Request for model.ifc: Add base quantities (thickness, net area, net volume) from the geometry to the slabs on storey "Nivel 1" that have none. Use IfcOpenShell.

First a look at what the model holds.

```python
import ifcopenshell
import ifcopenshell.util.element
import ifcopenshell.util.unit

model = ifcopenshell.open("model.ifc")
print(model.schema)
for unit_type in ("LENGTHUNIT", "AREAUNIT", "VOLUMEUNIT"):
    print(unit_type, ifcopenshell.util.unit.calculate_unit_scale(model, unit_type))
storey = next(s for s in model.by_type("IfcBuildingStorey") if s.Name == "Nivel 1")
slabs = [e for e in ifcopenshell.util.element.get_decomposition(storey) if e.is_a("IfcSlab")]
for e in sorted(slabs, key=lambda e: e.id()):
    print(e.id(), e.is_a(), e.Name, list(ifcopenshell.util.element.get_psets(e, qtos_only=True)), sep=" | ")
```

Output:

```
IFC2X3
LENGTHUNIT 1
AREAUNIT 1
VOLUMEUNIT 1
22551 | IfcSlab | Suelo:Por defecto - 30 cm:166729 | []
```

```python
import ifcopenshell
import ifcopenshell.api.pset
import ifcopenshell.geom
import ifcopenshell.util.element
import ifcopenshell.util.shape
import ifcopenshell.util.unit

model = ifcopenshell.open("model.ifc")
unit_scale = ifcopenshell.util.unit.calculate_unit_scale(model)
area_scale = ifcopenshell.util.unit.calculate_unit_scale(model, "AREAUNIT")
volume_scale = ifcopenshell.util.unit.calculate_unit_scale(model, "VOLUMEUNIT")
settings = ifcopenshell.geom.settings()

storey = next(s for s in model.by_type("IfcBuildingStorey") if s.Name == "Nivel 1")
slabs = [e for e in ifcopenshell.util.element.get_decomposition(storey) if e.is_a("IfcSlab")]

for e in sorted(slabs, key=lambda e: e.id()):
    if ifcopenshell.util.element.get_psets(e, qtos_only=True, should_inherit=False):
        continue
    # Geometry comes back in metres, in the element's own axes.
    shape = ifcopenshell.geom.create_shape(settings, e)
    values = {
        "Width": ifcopenshell.util.shape.get_z(shape.geometry) / unit_scale,
        "NetArea": ifcopenshell.util.shape.get_footprint_area(shape.geometry) / area_scale,
        "NetVolume": ifcopenshell.util.shape.get_volume(shape.geometry) / volume_scale,
    }
    qto = ifcopenshell.api.pset.add_qto(model, product=e, name="BaseQuantities")
    ifcopenshell.api.pset.edit_qto(model, qto=qto, properties=values)
    print(e.id(), {k: round(v, 3) for k, v in values.items()})

model.write("model_v2.ifc")
```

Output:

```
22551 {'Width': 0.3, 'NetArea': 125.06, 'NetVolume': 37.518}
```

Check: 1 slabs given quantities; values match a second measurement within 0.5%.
